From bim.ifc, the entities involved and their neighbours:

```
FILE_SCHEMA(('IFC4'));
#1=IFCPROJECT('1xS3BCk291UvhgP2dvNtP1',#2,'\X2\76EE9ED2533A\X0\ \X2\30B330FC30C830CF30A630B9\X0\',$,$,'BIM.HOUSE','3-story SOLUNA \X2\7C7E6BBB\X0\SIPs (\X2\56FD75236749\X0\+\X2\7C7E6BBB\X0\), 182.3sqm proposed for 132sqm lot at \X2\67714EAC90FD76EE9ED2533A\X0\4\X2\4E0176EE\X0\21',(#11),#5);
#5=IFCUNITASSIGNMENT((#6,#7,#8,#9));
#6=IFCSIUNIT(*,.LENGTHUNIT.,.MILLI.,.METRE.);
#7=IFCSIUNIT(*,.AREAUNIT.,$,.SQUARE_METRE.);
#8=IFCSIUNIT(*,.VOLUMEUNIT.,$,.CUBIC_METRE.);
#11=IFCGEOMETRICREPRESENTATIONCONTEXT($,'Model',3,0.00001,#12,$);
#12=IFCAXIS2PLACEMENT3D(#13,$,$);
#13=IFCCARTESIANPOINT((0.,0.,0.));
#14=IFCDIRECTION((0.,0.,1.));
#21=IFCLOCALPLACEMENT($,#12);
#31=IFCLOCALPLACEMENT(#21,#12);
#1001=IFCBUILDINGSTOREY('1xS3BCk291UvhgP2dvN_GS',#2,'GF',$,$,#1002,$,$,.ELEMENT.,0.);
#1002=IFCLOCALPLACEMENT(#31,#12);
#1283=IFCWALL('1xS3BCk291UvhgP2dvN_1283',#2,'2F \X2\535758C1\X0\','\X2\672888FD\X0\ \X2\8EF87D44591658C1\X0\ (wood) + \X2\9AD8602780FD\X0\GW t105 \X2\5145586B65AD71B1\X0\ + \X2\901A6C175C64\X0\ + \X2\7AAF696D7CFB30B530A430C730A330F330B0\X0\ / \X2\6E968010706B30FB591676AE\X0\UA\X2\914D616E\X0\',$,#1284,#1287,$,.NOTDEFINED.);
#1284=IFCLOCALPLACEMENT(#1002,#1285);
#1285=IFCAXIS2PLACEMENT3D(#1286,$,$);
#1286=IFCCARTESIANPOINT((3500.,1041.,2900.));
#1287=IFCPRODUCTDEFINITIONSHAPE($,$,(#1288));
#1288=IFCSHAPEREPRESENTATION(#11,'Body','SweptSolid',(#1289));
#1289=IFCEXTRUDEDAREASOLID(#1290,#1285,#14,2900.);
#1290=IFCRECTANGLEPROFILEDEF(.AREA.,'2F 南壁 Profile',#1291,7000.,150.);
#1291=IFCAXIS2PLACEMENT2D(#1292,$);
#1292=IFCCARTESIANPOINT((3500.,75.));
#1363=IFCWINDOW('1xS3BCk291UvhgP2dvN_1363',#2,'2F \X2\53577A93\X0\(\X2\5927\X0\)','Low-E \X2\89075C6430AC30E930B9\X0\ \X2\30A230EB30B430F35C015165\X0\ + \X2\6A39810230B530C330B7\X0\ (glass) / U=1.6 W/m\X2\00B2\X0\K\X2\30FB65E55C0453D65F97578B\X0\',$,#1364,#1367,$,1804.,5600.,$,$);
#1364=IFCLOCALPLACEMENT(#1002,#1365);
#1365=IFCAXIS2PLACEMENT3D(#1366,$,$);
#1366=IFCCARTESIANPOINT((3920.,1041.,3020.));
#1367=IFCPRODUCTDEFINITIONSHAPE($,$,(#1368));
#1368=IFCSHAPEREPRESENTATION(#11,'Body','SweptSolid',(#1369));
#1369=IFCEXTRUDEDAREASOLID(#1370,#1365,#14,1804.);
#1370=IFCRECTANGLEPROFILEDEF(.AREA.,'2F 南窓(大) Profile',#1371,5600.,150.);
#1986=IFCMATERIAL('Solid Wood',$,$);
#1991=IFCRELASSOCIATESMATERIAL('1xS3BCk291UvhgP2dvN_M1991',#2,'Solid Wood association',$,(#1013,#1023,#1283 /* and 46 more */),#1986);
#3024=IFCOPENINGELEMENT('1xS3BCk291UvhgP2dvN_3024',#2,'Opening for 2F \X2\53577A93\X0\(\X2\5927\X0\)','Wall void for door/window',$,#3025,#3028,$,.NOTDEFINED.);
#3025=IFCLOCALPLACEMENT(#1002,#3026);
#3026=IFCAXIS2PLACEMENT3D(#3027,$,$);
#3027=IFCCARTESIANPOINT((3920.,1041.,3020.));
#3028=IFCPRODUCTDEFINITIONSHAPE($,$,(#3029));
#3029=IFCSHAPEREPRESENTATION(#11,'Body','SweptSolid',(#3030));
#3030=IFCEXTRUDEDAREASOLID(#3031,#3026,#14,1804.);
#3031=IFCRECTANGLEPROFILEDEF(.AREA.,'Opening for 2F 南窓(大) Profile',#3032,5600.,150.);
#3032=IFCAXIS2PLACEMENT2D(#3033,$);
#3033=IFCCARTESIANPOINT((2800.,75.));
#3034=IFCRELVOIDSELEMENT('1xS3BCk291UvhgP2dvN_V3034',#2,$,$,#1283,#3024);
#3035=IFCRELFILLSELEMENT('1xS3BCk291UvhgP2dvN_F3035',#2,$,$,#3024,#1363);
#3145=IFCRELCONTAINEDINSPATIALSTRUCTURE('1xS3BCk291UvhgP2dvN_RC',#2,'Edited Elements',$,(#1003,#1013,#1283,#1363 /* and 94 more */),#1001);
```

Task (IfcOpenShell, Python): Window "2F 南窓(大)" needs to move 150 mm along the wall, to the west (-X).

```python
import ifcopenshell
import ifcopenshell.api.geometry
import ifcopenshell.util.placement

model = ifcopenshell.open("bim.ifc")

window = model.by_guid("1xS3BCk291UvhgP2dvN_1363")
opening = window.FillsVoids[0].RelatingOpeningElement
wall = opening.VoidsElements[0].RelatingBuildingElement

wall_matrix = ifcopenshell.util.placement.get_local_placement(wall.ObjectPlacement)
shift = wall_matrix[:3, 0] * -150.0
before = ifcopenshell.util.placement.get_local_placement(window.ObjectPlacement)[:3, 3].copy()

# The window is not placed relative to its opening, so move both.
for product in (opening, window):
    matrix = ifcopenshell.util.placement.get_local_placement(product.ObjectPlacement)
    matrix[:3, 3] += shift
    ifcopenshell.api.geometry.edit_object_placement(model, product=product, matrix=matrix, is_si=False)

after = ifcopenshell.util.placement.get_local_placement(window.ObjectPlacement)[:3, 3]
print("window moved by", (after - before).round(3) + 0.0)

model.write("bim-out.ifc")
```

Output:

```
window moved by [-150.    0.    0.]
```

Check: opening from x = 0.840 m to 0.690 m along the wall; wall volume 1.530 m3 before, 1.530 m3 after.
